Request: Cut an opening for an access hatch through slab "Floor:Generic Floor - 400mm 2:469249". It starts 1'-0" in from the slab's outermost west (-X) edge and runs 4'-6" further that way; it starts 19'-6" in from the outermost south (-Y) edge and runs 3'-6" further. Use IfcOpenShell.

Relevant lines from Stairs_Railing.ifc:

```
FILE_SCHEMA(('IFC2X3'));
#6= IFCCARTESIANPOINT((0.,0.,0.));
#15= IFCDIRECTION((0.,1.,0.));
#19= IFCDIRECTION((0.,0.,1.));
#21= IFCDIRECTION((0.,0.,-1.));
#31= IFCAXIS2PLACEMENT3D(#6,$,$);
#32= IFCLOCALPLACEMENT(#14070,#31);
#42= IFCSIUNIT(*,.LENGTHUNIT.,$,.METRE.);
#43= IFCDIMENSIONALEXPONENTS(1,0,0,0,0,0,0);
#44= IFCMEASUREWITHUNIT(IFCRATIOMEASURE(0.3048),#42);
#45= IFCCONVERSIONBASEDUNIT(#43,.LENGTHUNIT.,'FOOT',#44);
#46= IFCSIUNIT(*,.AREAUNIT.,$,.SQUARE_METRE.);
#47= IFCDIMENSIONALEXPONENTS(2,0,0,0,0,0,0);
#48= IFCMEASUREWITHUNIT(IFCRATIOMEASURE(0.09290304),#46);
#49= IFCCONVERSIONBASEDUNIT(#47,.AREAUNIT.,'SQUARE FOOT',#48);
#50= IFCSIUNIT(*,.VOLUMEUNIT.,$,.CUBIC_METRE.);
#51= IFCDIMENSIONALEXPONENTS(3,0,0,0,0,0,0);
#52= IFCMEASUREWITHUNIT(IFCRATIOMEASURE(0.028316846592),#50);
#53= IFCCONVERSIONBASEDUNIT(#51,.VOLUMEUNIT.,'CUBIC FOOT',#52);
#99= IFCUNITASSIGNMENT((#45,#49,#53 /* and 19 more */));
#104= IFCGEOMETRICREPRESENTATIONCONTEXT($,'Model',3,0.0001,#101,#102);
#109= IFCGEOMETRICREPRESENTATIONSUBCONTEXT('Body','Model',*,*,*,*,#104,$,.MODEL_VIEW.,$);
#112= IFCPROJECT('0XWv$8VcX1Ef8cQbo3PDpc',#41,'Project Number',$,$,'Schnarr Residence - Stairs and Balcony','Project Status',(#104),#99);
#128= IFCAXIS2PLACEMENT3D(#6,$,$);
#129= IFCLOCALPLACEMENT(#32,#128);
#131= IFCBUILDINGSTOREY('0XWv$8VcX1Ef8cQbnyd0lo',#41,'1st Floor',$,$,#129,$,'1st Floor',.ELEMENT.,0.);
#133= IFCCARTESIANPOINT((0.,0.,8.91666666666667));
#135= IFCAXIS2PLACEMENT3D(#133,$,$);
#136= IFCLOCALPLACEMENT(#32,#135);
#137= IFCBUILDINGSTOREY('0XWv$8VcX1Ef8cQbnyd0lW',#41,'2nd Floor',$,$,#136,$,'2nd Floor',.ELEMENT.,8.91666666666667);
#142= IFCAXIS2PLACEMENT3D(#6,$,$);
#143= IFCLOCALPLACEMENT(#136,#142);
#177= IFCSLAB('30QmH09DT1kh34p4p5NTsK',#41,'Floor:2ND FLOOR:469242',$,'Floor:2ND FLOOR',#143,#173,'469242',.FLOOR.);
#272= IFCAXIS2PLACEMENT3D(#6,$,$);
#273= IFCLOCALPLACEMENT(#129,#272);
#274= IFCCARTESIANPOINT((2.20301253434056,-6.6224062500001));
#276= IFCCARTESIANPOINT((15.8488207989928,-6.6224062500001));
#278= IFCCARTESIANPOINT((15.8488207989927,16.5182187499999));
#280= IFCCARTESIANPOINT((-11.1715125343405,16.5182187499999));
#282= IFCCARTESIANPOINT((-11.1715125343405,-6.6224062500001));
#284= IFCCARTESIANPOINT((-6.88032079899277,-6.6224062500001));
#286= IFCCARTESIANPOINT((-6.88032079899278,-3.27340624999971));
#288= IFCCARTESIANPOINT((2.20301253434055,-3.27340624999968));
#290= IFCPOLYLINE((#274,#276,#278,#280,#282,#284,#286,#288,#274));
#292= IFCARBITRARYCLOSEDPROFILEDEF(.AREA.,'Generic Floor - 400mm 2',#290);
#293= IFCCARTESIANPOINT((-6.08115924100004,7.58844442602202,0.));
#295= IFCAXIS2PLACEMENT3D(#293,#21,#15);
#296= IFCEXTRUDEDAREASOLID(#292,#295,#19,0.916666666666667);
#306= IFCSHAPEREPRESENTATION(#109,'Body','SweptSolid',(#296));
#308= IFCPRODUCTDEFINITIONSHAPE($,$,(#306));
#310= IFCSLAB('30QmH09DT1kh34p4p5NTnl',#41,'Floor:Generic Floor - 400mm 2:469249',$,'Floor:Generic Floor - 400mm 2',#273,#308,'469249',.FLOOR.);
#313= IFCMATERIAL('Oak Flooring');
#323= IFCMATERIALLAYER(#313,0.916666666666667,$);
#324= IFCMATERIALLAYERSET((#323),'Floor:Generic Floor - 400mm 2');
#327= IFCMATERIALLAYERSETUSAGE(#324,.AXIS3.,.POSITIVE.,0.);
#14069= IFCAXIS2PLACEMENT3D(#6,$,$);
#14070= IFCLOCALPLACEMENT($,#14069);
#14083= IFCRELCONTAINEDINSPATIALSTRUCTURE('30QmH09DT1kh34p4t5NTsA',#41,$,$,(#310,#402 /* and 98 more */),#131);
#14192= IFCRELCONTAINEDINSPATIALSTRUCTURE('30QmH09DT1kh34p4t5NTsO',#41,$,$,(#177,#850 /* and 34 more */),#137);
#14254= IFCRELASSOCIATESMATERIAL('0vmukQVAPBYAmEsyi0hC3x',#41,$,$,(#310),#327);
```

```python
import numpy as np
import ifcopenshell
import ifcopenshell.api.feature
import ifcopenshell.api.geometry
import ifcopenshell.api.root
import ifcopenshell.geom
import ifcopenshell.util.placement
import ifcopenshell.util.representation
import ifcopenshell.util.shape
import ifcopenshell.util.unit

model = ifcopenshell.open("Stairs_Railing.ifc")
unit_scale = ifcopenshell.util.unit.calculate_unit_scale(model)
settings = ifcopenshell.geom.settings()


def volume(element):
    """Net volume in cubic metres, openings subtracted."""
    shape = ifcopenshell.geom.create_shape(settings, element)
    return ifcopenshell.util.shape.get_volume(shape.geometry)


slab = model.by_guid("30QmH09DT1kh34p4p5NTnl")
before = volume(slab)

# Extent in the slab's own axes, in metres. The edges named are its -X and -Y sides.
slab_shape = ifcopenshell.geom.create_shape(settings, slab)
vertices = ifcopenshell.util.shape.get_vertices(slab_shape.geometry)
x_min, y_min, bottom = vertices.min(axis=0)
top = vertices[:, 2].max()

opening = ifcopenshell.api.root.create_entity(model, ifc_class="IfcOpeningElement", name="Access hatch opening")
context = ifcopenshell.util.representation.get_context(model, "Model", "Body", "MODEL_VIEW")
width, depth = 1.3716, 1.0668
outline = [(0.0, 0.0), (width, 0.0), (width, depth), (0.0, depth), (0.0, 0.0)]
# Overshoot both faces by 50 mm so the cut is clean.
shape = ifcopenshell.api.geometry.add_slab_representation(
    model, context=context, depth=top - bottom + 0.1, polyline=outline
)
ifcopenshell.api.geometry.assign_representation(model, product=opening, representation=shape)

matrix = ifcopenshell.util.placement.get_local_placement(slab.ObjectPlacement)
matrix[:, 3] = matrix @ np.append(np.array([x_min + 0.3048, y_min + 5.9436, bottom - 0.05]) / unit_scale, 1.0)
ifcopenshell.api.geometry.edit_object_placement(model, product=opening, matrix=matrix, is_si=False)
ifcopenshell.api.feature.add_feature(model, feature=opening, element=slab)

after = volume(slab)

print(f"slab volume {before:.3f} -> {after:.3f} m3")

model.write("Stairs_Railing_v2.ifc")
```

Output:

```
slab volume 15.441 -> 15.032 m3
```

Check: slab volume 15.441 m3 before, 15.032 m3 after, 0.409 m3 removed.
